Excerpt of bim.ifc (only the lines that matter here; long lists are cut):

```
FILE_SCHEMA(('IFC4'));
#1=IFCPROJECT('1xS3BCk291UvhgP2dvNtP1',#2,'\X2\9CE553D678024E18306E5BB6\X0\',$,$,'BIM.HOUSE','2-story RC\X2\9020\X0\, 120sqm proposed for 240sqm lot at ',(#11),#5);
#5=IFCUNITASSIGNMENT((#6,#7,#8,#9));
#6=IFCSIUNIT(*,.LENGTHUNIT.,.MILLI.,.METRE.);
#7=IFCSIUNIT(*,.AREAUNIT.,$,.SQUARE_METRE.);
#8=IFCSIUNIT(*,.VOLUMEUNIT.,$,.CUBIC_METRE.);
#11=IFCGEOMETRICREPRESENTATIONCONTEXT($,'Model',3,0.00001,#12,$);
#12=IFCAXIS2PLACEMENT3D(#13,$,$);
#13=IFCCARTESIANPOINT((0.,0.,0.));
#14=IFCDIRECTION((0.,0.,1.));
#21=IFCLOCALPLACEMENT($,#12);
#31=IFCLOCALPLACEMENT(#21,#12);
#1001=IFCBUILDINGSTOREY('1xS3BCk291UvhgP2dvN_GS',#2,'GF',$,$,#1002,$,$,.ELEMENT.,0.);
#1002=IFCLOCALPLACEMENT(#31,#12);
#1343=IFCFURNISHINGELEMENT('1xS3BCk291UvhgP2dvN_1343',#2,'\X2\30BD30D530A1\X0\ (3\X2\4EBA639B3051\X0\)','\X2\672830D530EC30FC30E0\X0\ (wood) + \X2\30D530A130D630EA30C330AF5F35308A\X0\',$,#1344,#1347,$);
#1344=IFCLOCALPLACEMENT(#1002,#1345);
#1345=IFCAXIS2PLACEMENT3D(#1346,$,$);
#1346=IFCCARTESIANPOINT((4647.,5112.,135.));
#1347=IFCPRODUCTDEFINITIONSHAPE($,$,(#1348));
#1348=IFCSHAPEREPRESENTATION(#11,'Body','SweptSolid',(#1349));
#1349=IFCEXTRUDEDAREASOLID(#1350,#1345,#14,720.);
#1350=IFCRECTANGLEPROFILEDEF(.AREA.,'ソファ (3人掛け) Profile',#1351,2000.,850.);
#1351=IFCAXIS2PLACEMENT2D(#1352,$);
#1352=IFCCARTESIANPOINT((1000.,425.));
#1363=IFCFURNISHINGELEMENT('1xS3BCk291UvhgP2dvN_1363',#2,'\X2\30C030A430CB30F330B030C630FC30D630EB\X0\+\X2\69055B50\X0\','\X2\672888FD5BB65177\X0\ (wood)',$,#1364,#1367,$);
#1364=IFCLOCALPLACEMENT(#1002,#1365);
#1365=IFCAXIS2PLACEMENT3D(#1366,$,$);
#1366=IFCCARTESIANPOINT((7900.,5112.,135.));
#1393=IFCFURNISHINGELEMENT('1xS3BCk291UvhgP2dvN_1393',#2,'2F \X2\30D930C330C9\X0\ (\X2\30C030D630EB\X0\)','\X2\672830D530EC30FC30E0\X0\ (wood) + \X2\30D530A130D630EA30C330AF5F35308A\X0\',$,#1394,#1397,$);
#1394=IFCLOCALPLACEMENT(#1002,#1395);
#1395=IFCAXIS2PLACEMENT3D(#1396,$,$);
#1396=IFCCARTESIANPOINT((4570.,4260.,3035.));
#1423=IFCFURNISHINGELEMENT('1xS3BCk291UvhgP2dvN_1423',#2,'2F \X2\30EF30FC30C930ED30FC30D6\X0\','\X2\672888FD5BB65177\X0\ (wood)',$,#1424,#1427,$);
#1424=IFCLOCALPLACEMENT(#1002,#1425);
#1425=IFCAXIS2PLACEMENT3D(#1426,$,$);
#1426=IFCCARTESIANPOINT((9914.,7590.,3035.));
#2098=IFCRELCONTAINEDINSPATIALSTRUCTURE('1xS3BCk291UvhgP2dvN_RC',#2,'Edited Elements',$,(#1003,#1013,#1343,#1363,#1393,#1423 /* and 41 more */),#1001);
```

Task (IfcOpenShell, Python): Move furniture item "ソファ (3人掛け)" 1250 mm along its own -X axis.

```python
import ifcopenshell
import ifcopenshell.api.geometry
import ifcopenshell.util.placement

model = ifcopenshell.open("bim.ifc")

item = model.by_guid("1xS3BCk291UvhgP2dvN_1343")
matrix = ifcopenshell.util.placement.get_local_placement(item.ObjectPlacement)
matrix[:3, 3] -= matrix[:3, 0] * 1250.0
ifcopenshell.api.geometry.edit_object_placement(model, product=item, matrix=matrix, is_si=False)

print(ifcopenshell.util.placement.get_local_placement(item.ObjectPlacement).round(3) + 0.0)

model.write("bim_v2.ifc")
```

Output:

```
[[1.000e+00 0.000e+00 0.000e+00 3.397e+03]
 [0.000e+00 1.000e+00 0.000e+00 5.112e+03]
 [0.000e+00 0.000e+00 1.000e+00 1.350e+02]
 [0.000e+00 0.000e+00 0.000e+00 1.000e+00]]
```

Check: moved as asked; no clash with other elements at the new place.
